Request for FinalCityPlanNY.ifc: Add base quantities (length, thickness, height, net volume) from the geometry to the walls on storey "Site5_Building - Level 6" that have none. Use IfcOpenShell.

First a look at what the model holds.

```python
import ifcopenshell
import ifcopenshell.util.element
import ifcopenshell.util.unit

model = ifcopenshell.open("FinalCityPlanNY.ifc")
print(model.schema)
for unit_type in ("LENGTHUNIT", "AREAUNIT", "VOLUMEUNIT"):
    print(unit_type, ifcopenshell.util.unit.calculate_unit_scale(model, unit_type))
storey = next(s for s in model.by_type("IfcBuildingStorey") if s.Name == "Site5_Building - Level 6")
walls = [e for e in ifcopenshell.util.element.get_decomposition(storey) if e.is_a("IfcWall")]
for e in sorted(walls, key=lambda e: e.id()):
    print(e.id(), e.is_a(), e.Name, list(ifcopenshell.util.element.get_psets(e, qtos_only=True)), sep=" | ")
```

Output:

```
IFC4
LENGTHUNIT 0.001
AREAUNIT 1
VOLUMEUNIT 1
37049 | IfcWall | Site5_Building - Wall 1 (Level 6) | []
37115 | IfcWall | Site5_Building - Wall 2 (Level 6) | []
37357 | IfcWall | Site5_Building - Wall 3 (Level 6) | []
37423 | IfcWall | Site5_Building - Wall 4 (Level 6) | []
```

```python
import ifcopenshell
import ifcopenshell.api.pset
import ifcopenshell.geom
import ifcopenshell.util.element
import ifcopenshell.util.shape
import ifcopenshell.util.unit

model = ifcopenshell.open("FinalCityPlanNY.ifc")
unit_scale = ifcopenshell.util.unit.calculate_unit_scale(model)
volume_scale = ifcopenshell.util.unit.calculate_unit_scale(model, "VOLUMEUNIT")
settings = ifcopenshell.geom.settings()

storey = next(s for s in model.by_type("IfcBuildingStorey") if s.Name == "Site5_Building - Level 6")
walls = [e for e in ifcopenshell.util.element.get_decomposition(storey) if e.is_a("IfcWall")]

for e in sorted(walls, key=lambda e: e.id()):
    if ifcopenshell.util.element.get_psets(e, qtos_only=True, should_inherit=False):
        continue
    # Geometry comes back in metres, in the element's own axes.
    shape = ifcopenshell.geom.create_shape(settings, e)
    values = {
        "Length": ifcopenshell.util.shape.get_x(shape.geometry) / unit_scale,
        "Width": ifcopenshell.util.shape.get_y(shape.geometry) / unit_scale,
        "Height": ifcopenshell.util.shape.get_z(shape.geometry) / unit_scale,
        "NetVolume": ifcopenshell.util.shape.get_volume(shape.geometry) / volume_scale,
    }
    qto = ifcopenshell.api.pset.add_qto(model, product=e, name="Qto_WallBaseQuantities")
    ifcopenshell.api.pset.edit_qto(model, qto=qto, properties=values)
    print(e.id(), {k: round(v, 3) for k, v in values.items()})

model.write("FinalCityPlanNY_edited.ifc")
```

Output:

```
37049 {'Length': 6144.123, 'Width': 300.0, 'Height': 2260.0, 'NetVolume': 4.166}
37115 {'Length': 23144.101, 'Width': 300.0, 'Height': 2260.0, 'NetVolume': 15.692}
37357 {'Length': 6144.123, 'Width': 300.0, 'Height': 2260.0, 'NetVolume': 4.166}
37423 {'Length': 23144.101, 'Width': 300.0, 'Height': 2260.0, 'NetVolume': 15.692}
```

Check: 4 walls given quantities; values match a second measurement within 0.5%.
